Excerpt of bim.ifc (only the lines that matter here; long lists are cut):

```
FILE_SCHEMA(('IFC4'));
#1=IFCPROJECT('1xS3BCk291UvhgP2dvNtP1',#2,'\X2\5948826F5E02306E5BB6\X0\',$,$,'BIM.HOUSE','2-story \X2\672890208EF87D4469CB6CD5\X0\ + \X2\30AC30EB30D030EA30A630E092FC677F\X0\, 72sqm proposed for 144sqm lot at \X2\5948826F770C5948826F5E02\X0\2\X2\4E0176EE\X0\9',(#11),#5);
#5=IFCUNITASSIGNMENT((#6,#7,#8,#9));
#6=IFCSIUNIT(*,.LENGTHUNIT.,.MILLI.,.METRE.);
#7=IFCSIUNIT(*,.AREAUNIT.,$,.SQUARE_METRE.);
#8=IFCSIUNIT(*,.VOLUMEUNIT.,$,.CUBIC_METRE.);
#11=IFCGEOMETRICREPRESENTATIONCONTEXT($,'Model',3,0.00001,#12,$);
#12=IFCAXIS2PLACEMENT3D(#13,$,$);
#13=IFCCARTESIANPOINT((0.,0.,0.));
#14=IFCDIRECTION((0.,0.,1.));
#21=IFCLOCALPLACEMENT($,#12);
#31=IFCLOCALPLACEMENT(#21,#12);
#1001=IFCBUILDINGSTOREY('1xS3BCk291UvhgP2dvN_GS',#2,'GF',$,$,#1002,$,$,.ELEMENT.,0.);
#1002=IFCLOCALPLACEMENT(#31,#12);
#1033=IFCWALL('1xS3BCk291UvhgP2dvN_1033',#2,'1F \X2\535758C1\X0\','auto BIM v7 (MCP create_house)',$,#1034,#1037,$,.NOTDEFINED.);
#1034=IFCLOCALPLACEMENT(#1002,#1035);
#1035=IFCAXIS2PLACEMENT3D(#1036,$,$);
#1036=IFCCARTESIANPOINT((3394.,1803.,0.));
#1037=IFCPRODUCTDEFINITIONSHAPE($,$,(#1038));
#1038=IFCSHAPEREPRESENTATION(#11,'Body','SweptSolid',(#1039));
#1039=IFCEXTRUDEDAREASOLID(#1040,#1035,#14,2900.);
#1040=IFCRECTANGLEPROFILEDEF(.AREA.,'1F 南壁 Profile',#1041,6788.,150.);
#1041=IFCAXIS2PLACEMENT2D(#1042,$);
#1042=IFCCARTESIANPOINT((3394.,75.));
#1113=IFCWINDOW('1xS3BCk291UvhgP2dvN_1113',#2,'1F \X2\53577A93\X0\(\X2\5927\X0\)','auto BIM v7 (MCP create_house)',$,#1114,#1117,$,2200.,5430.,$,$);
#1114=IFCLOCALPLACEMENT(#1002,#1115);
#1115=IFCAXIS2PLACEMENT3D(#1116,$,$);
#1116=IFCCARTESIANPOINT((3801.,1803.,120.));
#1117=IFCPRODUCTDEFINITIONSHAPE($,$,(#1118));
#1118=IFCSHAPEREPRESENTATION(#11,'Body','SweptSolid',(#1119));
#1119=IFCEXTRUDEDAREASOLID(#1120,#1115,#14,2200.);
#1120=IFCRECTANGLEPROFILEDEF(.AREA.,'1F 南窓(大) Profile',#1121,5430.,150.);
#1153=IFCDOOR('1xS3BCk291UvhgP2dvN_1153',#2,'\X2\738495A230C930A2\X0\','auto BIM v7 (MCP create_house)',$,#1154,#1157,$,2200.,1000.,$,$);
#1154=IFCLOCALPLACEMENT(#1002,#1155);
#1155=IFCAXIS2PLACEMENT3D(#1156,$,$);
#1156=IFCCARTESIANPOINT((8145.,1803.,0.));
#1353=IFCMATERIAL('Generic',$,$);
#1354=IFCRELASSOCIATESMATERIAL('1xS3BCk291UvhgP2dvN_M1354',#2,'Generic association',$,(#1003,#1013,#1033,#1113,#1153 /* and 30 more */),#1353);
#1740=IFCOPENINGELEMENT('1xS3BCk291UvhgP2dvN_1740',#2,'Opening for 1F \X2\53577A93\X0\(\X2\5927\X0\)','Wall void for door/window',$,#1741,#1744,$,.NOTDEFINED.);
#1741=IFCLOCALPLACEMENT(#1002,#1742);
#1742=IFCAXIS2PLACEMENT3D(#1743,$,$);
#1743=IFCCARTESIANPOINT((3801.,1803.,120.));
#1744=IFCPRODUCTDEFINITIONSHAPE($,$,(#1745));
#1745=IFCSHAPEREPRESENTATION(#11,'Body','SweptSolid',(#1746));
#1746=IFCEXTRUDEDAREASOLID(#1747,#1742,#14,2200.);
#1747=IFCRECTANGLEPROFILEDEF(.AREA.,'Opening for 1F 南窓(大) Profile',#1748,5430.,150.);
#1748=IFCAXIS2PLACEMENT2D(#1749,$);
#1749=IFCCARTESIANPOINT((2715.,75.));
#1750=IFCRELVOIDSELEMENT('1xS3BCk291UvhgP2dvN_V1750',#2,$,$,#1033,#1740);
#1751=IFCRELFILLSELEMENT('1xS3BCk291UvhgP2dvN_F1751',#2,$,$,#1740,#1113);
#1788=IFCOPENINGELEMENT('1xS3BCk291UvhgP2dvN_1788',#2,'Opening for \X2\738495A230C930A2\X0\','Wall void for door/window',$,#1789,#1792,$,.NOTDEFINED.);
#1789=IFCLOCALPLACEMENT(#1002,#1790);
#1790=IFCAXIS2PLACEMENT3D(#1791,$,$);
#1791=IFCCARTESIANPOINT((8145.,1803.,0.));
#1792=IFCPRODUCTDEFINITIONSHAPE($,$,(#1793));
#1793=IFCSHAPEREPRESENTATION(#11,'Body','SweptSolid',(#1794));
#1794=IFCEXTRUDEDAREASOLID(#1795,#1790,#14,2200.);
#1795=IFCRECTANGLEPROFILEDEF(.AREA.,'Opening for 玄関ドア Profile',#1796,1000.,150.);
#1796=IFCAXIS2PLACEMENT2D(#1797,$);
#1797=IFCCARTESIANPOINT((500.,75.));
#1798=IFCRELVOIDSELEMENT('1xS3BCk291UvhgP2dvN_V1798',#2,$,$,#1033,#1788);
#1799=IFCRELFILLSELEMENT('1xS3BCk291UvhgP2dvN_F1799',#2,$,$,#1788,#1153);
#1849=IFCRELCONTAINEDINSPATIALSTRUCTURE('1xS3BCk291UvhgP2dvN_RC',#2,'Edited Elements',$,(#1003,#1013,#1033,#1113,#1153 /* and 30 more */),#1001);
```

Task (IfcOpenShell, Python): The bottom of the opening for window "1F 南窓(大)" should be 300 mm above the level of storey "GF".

```python
import numpy as np
import ifcopenshell
import ifcopenshell.api.geometry
import ifcopenshell.geom
import ifcopenshell.util.element
import ifcopenshell.util.placement
import ifcopenshell.util.shape
import ifcopenshell.util.unit

model = ifcopenshell.open("bim.ifc")
unit_scale = ifcopenshell.util.unit.calculate_unit_scale(model)

window = model.by_id(1113)
opening = window.FillsVoids[0].RelatingOpeningElement
storey = ifcopenshell.util.element.get_container(window, ifc_class="IfcBuildingStorey")
level = ifcopenshell.util.placement.get_local_placement(storey.ObjectPlacement)[2, 3]

# The opening's origin need not be at the sill, so measure its lowest point.
shape = ifcopenshell.geom.create_shape(ifcopenshell.geom.settings(), opening)
bottom = ifcopenshell.util.shape.get_shape_bottom_elevation(shape, shape.geometry) / unit_scale
dz = level + 300.0 - bottom

shift = np.array([0.0, 0.0, dz])
# The window is not placed relative to its opening, so move both.
for product in (opening, window):
    matrix = ifcopenshell.util.placement.get_local_placement(product.ObjectPlacement)
    matrix[:3, 3] += shift
    ifcopenshell.api.geometry.edit_object_placement(model, product=product, matrix=matrix, is_si=False)

print(f"moved by {dz * unit_scale:+.3f} m")

model.write("bim_rev.ifc")
```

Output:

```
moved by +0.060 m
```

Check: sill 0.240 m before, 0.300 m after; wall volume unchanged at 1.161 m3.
